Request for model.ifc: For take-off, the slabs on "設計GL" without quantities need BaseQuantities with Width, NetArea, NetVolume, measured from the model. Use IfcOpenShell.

First a look at what the model holds.

```python
import ifcopenshell
import ifcopenshell.util.element
import ifcopenshell.util.unit

model = ifcopenshell.open("model.ifc")
print(model.schema)
for unit_type in ("LENGTHUNIT", "AREAUNIT", "VOLUMEUNIT"):
    print(unit_type, ifcopenshell.util.unit.calculate_unit_scale(model, unit_type))
storey = next(s for s in model.by_type("IfcBuildingStorey") if s.Name == "設計GL")
slabs = [e for e in ifcopenshell.util.element.get_decomposition(storey) if e.is_a("IfcSlab")]
for e in sorted(slabs, key=lambda e: e.id()):
    print(e.id(), e.is_a(), e.Name, list(ifcopenshell.util.element.get_psets(e, qtos_only=True)), sep=" | ")
```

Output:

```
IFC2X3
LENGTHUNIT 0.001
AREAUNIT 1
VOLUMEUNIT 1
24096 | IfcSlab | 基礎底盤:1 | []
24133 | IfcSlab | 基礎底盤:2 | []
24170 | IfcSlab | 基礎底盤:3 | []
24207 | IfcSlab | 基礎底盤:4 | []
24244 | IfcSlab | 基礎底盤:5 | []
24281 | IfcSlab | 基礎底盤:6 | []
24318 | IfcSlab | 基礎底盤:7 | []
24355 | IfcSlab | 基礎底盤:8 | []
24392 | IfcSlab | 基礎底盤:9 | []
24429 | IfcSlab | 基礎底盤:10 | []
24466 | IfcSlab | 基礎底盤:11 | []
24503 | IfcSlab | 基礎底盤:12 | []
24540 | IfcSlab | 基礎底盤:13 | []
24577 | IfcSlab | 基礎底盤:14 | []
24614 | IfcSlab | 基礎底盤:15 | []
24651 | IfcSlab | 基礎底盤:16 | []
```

```python
import ifcopenshell
import ifcopenshell.api.pset
import ifcopenshell.geom
import ifcopenshell.util.element
import ifcopenshell.util.shape
import ifcopenshell.util.unit

model = ifcopenshell.open("model.ifc")
unit_scale = ifcopenshell.util.unit.calculate_unit_scale(model)
area_scale = ifcopenshell.util.unit.calculate_unit_scale(model, "AREAUNIT")
volume_scale = ifcopenshell.util.unit.calculate_unit_scale(model, "VOLUMEUNIT")
settings = ifcopenshell.geom.settings()

storey = next(s for s in model.by_type("IfcBuildingStorey") if s.Name == "設計GL")
slabs = [e for e in ifcopenshell.util.element.get_decomposition(storey) if e.is_a("IfcSlab")]

for e in sorted(slabs, key=lambda e: e.id()):
    if ifcopenshell.util.element.get_psets(e, qtos_only=True, should_inherit=False):
        continue
    # Geometry comes back in metres, in the element's own axes.
    shape = ifcopenshell.geom.create_shape(settings, e)
    values = {
        "Width": ifcopenshell.util.shape.get_z(shape.geometry) / unit_scale,
        "NetArea": ifcopenshell.util.shape.get_footprint_area(shape.geometry) / area_scale,
        "NetVolume": ifcopenshell.util.shape.get_volume(shape.geometry) / volume_scale,
    }
    qto = ifcopenshell.api.pset.add_qto(model, product=e, name="BaseQuantities")
    ifcopenshell.api.pset.edit_qto(model, qto=qto, properties=values)
    print(e.id(), {k: round(v, 3) for k, v in values.items()})

model.write("model-out.ifc")
```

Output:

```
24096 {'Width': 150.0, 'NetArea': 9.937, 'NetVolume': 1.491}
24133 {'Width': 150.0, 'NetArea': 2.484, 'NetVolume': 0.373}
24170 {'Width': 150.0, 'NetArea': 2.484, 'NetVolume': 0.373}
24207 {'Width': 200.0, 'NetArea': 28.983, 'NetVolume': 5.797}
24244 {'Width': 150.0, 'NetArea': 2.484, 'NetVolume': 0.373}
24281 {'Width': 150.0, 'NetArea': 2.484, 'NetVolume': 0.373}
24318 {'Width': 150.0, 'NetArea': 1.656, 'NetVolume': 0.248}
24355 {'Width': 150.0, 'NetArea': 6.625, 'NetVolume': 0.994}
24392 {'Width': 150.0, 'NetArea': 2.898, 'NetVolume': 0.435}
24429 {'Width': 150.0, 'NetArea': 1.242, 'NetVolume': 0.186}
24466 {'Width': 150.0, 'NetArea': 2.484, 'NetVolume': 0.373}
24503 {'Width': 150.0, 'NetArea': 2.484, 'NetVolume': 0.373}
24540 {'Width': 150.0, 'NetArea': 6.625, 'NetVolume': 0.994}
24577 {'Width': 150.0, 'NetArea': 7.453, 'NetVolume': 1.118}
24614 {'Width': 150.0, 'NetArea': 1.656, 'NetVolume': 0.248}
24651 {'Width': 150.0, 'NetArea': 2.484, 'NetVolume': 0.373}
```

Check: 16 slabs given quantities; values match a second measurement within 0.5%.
